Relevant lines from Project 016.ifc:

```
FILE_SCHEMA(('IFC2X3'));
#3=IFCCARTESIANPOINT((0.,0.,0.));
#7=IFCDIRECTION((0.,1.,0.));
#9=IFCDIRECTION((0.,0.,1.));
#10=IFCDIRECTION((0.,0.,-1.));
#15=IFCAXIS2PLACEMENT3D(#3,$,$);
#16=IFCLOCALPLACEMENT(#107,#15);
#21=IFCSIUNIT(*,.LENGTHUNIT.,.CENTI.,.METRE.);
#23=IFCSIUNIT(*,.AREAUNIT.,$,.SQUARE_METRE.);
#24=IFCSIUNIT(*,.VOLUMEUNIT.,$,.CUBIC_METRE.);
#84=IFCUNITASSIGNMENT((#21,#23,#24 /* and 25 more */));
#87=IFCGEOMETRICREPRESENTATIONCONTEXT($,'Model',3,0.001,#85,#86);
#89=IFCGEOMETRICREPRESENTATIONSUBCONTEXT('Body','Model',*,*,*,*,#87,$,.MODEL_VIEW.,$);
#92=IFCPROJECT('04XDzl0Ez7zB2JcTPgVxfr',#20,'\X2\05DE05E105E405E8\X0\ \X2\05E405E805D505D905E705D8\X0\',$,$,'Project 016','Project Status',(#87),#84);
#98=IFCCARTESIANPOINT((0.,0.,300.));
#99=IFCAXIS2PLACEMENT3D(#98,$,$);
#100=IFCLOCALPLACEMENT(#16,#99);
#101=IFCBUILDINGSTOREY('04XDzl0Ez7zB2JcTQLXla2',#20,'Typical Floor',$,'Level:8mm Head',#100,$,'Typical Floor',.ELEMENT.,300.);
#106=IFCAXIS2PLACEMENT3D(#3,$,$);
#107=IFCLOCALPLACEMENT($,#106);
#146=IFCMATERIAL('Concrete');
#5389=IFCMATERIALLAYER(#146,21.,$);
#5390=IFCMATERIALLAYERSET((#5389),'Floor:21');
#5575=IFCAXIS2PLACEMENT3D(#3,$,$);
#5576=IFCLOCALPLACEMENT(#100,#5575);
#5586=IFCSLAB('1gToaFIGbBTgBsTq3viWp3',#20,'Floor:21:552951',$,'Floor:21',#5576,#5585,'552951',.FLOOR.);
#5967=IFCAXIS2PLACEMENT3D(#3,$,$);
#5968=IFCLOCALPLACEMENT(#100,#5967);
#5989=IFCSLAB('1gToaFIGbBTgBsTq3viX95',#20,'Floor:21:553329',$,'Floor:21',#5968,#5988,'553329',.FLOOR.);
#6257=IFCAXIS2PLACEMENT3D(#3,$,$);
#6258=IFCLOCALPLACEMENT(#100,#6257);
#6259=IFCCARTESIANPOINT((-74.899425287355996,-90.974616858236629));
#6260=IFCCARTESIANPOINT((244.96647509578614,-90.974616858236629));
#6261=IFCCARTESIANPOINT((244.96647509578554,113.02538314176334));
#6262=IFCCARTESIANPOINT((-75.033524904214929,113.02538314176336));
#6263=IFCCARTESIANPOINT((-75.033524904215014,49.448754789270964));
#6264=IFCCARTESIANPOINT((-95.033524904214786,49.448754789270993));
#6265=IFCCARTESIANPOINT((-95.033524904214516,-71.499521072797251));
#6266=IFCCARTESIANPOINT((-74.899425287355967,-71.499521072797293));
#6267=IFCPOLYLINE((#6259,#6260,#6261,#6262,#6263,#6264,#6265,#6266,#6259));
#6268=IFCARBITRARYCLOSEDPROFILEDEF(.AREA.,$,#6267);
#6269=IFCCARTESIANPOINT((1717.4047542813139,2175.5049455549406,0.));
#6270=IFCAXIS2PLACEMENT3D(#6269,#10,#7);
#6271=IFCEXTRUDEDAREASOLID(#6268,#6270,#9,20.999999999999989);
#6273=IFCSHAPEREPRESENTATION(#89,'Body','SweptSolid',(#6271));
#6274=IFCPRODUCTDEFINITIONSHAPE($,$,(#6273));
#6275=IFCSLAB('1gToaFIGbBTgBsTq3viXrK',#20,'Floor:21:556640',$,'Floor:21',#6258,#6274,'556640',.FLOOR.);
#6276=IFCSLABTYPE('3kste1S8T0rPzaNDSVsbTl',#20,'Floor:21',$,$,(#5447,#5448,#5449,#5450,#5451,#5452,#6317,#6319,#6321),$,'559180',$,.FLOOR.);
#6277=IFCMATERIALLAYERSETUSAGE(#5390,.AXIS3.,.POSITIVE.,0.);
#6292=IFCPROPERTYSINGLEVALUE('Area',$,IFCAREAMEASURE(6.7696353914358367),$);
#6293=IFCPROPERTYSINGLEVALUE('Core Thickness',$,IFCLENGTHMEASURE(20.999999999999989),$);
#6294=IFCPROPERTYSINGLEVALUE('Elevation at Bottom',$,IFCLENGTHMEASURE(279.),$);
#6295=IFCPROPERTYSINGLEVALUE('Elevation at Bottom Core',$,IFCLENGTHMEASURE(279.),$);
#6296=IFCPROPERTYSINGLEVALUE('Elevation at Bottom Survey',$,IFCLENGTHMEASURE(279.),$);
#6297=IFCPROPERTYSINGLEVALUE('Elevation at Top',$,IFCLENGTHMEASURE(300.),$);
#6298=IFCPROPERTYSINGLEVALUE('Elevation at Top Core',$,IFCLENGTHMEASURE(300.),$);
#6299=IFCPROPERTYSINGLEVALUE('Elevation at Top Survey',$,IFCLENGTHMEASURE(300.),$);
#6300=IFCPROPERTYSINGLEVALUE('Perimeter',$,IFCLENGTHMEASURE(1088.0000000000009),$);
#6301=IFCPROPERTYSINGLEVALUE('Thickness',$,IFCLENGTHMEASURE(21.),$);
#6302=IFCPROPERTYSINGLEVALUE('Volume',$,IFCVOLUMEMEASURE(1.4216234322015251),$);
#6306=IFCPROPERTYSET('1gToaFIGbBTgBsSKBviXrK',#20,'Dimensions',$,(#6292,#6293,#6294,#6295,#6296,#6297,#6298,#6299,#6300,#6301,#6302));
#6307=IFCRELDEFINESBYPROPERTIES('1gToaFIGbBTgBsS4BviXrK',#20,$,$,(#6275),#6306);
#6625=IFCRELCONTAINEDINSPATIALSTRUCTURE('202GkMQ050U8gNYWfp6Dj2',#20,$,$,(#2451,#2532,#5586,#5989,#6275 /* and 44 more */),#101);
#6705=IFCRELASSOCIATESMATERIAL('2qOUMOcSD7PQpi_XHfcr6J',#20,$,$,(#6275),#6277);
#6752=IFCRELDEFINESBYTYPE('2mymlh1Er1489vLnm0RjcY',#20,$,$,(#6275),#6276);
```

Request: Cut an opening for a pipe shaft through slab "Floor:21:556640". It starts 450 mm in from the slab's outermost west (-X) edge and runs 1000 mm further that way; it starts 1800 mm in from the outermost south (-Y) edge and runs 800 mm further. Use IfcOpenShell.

```python
import numpy as np
import ifcopenshell
import ifcopenshell.api.feature
import ifcopenshell.api.geometry
import ifcopenshell.api.pset
import ifcopenshell.api.root
import ifcopenshell.geom
import ifcopenshell.util.element
import ifcopenshell.util.placement
import ifcopenshell.util.representation
import ifcopenshell.util.shape
import ifcopenshell.util.unit

model = ifcopenshell.open("Project 016.ifc")
unit_scale = ifcopenshell.util.unit.calculate_unit_scale(model)
area_scale = ifcopenshell.util.unit.calculate_unit_scale(model, "AREAUNIT")
volume_scale = ifcopenshell.util.unit.calculate_unit_scale(model, "VOLUMEUNIT")
settings = ifcopenshell.geom.settings()


def volume(element):
    """Net volume in cubic metres, openings subtracted."""
    shape = ifcopenshell.geom.create_shape(settings, element)
    return ifcopenshell.util.shape.get_volume(shape.geometry)


slab = model.by_guid("1gToaFIGbBTgBsTq3viXrK")
before = volume(slab)

# Extent in the slab's own axes, in metres. The edges named are its -X and -Y sides.
slab_shape = ifcopenshell.geom.create_shape(settings, slab)
vertices = ifcopenshell.util.shape.get_vertices(slab_shape.geometry)
x_min, y_min, bottom = vertices.min(axis=0)
top = vertices[:, 2].max()

opening = ifcopenshell.api.root.create_entity(model, ifc_class="IfcOpeningElement", name="Pipe shaft opening")
context = ifcopenshell.util.representation.get_context(model, "Model", "Body", "MODEL_VIEW")
width, depth = 1, 0.8
outline = [(0.0, 0.0), (width, 0.0), (width, depth), (0.0, depth), (0.0, 0.0)]
# Overshoot both faces by 50 mm so the cut is clean.
shape = ifcopenshell.api.geometry.add_slab_representation(
    model, context=context, depth=top - bottom + 0.1, polyline=outline
)
ifcopenshell.api.geometry.assign_representation(model, product=opening, representation=shape)

matrix = ifcopenshell.util.placement.get_local_placement(slab.ObjectPlacement)
matrix[:, 3] = matrix @ np.append(np.array([x_min + 0.45, y_min + 1.8, bottom - 0.05]) / unit_scale, 1.0)
ifcopenshell.api.geometry.edit_object_placement(model, product=opening, matrix=matrix, is_si=False)
ifcopenshell.api.feature.add_feature(model, feature=opening, element=slab)

after = volume(slab)

# Update the slab's stored quantities.
pset = model.by_id(ifcopenshell.util.element.get_pset(slab, "Dimensions", should_inherit=False)["id"])
ifcopenshell.api.pset.edit_pset(model, pset=pset, properties={
    "Area": model.create_entity("IfcAreaMeasure", after / (top - bottom) / area_scale),
    "Volume": model.create_entity("IfcVolumeMeasure", after / volume_scale),
})

print(f"slab volume {before:.3f} -> {after:.3f} m3")

model.write("Project 016_updated.ifc")
```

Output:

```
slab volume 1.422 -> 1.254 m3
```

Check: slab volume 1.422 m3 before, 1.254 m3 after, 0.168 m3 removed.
